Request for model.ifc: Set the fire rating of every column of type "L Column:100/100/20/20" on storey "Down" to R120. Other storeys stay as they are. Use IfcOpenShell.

First a look at what the model holds.

```python
import ifcopenshell
import ifcopenshell.util.element

model = ifcopenshell.open("model.ifc")
print(model.schema)
storey = next(s for s in model.by_type("IfcBuildingStorey") if s.Name == "Down")
columns = [e for e in ifcopenshell.util.element.get_decomposition(storey) if e.is_a("IfcColumn")]
seen = {}
for e in columns:
    element_type = ifcopenshell.util.element.get_type(e)
    key = (element_type.Name if element_type != e and element_type else None, ifcopenshell.util.element.get_pset(e, "Pset_ColumnCommon", "FireRating"))
    seen[key] = seen.get(key, 0) + 1
for (name, value), count in sorted(seen.items(), key=str):
    print(count, "x", name, "|", value)
```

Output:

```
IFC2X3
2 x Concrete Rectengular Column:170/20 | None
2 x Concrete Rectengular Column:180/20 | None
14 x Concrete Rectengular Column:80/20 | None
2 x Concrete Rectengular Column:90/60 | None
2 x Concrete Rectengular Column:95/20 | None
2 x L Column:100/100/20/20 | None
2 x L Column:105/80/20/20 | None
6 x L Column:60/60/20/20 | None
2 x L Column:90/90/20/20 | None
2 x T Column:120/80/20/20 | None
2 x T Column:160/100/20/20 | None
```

```python
import ifcopenshell
import ifcopenshell.api.pset
import ifcopenshell.util.element

model = ifcopenshell.open("model.ifc")

storey = next(s for s in model.by_type("IfcBuildingStorey") if s.Name == "Down")
columns = [e for e in ifcopenshell.util.element.get_decomposition(storey) if e.is_a("IfcColumn")]

count = 0
for e in columns:
    element_type = ifcopenshell.util.element.get_type(e)
    if element_type in (None, e) or element_type.Name != "L Column:100/100/20/20":
        continue
    # add_pset returns the element's existing set when there is one.
    pset = ifcopenshell.api.pset.add_pset(model, product=e, name="Pset_ColumnCommon")
    ifcopenshell.api.pset.edit_pset(model, pset=pset, properties={"FireRating": "R120"})
    count += 1

print(count, "columns updated")

model.write("model_v2.ifc")
```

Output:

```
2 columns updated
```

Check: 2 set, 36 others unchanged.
